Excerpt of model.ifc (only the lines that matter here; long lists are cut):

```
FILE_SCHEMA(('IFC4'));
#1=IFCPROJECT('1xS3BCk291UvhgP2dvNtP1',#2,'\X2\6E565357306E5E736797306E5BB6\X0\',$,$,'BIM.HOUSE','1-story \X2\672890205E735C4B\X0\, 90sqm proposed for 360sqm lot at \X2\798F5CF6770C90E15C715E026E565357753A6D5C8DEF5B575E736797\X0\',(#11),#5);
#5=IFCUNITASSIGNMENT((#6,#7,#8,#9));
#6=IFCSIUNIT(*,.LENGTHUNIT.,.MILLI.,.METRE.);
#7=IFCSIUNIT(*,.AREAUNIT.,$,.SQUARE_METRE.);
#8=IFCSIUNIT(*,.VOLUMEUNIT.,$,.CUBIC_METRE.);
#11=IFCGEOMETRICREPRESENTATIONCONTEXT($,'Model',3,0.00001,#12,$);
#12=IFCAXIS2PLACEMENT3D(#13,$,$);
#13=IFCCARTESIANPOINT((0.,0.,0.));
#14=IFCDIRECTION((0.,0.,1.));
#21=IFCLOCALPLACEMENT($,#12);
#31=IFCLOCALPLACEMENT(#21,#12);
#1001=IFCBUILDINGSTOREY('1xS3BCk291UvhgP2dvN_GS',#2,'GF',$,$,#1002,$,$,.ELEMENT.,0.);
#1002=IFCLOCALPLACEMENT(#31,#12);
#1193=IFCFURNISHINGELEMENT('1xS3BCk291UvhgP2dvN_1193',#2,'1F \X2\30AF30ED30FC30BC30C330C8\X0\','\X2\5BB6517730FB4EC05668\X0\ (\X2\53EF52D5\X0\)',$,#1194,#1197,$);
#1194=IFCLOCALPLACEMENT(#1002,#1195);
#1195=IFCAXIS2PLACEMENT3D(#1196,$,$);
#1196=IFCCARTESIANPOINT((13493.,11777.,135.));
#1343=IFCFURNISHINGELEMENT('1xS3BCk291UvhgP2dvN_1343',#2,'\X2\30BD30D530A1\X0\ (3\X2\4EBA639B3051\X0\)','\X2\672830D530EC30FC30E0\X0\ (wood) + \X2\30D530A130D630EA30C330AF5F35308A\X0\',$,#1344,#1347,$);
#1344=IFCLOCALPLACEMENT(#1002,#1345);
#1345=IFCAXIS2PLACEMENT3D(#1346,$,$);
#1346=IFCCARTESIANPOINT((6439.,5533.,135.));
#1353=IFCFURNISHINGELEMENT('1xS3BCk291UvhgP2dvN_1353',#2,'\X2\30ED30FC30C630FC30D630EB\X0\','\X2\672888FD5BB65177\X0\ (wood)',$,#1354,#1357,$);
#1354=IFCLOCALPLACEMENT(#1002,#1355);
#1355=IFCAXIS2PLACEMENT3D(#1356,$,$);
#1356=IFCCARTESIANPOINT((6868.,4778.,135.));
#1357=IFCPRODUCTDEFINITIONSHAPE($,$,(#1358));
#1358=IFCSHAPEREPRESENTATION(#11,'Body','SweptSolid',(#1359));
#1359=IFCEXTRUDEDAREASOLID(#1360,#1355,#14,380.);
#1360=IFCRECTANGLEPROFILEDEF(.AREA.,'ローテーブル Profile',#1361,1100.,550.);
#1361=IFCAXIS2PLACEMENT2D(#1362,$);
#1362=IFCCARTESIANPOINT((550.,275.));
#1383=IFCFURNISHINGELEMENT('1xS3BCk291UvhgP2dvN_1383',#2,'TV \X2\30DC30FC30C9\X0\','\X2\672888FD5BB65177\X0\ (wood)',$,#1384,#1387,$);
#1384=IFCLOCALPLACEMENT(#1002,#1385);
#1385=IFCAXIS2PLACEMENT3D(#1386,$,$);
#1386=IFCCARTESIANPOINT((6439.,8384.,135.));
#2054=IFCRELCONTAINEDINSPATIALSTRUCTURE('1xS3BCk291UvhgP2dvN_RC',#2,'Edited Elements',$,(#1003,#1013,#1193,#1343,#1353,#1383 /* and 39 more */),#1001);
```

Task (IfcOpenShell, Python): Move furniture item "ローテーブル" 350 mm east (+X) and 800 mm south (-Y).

```python
import ifcopenshell
import ifcopenshell.api.geometry
import ifcopenshell.util.placement
import ifcopenshell.util.unit

model = ifcopenshell.open("model.ifc")
unit_scale = ifcopenshell.util.unit.calculate_unit_scale(model)

item = model.by_guid("1xS3BCk291UvhgP2dvN_1353")
matrix = ifcopenshell.util.placement.get_local_placement(item.ObjectPlacement)
matrix[0, 3] += 0.35 / unit_scale
matrix[1, 3] -= 0.8 / unit_scale
ifcopenshell.api.geometry.edit_object_placement(model, product=item, matrix=matrix, is_si=False)

print(ifcopenshell.util.placement.get_local_placement(item.ObjectPlacement).round(3) + 0.0)

model.write("model_v2.ifc")
```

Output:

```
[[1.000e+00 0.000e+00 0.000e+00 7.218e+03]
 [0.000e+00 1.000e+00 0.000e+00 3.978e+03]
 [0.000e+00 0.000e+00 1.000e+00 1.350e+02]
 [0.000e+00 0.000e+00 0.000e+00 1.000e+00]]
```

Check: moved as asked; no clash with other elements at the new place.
